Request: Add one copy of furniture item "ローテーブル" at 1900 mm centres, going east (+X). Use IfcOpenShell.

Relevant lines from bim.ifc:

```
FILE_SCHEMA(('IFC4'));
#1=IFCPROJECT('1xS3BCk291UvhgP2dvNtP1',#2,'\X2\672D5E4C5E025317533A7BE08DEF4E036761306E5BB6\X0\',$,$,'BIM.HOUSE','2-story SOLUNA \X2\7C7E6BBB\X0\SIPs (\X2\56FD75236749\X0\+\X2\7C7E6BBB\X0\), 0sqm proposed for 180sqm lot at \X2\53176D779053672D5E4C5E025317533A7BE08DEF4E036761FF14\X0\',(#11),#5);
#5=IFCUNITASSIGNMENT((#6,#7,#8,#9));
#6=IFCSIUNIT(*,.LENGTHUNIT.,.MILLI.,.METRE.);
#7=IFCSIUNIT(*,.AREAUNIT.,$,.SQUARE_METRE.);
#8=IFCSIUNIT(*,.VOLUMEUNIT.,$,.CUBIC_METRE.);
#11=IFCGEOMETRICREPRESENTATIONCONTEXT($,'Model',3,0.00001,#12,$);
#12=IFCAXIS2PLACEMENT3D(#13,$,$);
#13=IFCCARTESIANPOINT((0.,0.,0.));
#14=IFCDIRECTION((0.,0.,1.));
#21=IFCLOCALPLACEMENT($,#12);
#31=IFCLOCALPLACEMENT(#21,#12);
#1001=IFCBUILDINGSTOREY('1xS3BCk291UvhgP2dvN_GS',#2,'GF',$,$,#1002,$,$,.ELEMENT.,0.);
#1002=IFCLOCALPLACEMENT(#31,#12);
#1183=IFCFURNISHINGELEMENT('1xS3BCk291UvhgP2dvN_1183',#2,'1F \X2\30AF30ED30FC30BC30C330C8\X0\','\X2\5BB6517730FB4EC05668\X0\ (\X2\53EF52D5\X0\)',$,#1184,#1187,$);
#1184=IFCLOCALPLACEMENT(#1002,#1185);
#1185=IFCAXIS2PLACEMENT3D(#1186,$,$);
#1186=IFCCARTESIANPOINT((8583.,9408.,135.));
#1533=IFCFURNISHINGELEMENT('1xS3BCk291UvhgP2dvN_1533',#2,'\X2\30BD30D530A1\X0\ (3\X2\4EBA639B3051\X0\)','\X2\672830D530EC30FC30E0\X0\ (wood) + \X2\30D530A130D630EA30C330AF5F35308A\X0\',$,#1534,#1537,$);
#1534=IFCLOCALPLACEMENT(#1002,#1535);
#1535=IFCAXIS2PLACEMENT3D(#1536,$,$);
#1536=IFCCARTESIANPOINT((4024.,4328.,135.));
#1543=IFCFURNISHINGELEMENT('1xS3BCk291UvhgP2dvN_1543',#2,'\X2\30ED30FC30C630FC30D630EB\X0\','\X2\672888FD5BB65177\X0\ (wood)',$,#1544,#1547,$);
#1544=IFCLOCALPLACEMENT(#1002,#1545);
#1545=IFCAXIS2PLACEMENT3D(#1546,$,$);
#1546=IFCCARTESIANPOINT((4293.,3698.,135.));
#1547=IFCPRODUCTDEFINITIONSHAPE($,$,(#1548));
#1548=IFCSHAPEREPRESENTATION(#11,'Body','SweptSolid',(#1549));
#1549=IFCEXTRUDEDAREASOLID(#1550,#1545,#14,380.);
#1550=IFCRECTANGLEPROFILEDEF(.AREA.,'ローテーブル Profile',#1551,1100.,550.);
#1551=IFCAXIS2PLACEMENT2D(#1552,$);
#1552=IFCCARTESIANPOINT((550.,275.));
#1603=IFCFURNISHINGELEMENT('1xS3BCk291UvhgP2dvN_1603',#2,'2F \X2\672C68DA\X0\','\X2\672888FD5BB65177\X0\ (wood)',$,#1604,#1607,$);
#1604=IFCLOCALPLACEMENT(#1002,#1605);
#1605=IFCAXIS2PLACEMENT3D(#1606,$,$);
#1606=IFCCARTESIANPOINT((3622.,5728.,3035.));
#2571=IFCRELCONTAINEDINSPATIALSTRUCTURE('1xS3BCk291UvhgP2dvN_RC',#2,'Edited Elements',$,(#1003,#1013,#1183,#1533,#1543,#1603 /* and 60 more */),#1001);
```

```python
import numpy as np
import ifcopenshell
import ifcopenshell.api.geometry
import ifcopenshell.api.root
import ifcopenshell.util.element
import ifcopenshell.util.placement

model = ifcopenshell.open("bim.ifc")


def reuse_history(source, copy):
    """copy_class also copies each property set's owner history, people and application; keep the originals."""
    for rel in copy.IsDefinedBy:
        if rel.is_a("IfcRelDefinesByProperties") and (history := rel.RelatingPropertyDefinition.OwnerHistory):
            rel.RelatingPropertyDefinition.OwnerHistory = source.OwnerHistory
            ifcopenshell.util.element.remove_deep2(model, history)


source = model.by_guid("1xS3BCk291UvhgP2dvN_1543")
base = ifcopenshell.util.placement.get_local_placement(source.ObjectPlacement)
step = np.array([1.0, 0.0, 0.0]) * 1900.0

for i in range(1, 2):
    copy = ifcopenshell.api.root.copy_class(model, product=source)
    copy.Representation = ifcopenshell.util.element.copy_deep(
        model, source.Representation, exclude=["IfcGeometricRepresentationContext", "IfcRepresentationMap"]
    )
    reuse_history(source, copy)
    matrix = base.copy()
    matrix[:3, 3] += i * step
    print("added at", matrix[:3, 3].round(3) + 0.0)
    ifcopenshell.api.geometry.edit_object_placement(model, product=copy, matrix=matrix, is_si=False)

model.write("bim_updated.ifc")
```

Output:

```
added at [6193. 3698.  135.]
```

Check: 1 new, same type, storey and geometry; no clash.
